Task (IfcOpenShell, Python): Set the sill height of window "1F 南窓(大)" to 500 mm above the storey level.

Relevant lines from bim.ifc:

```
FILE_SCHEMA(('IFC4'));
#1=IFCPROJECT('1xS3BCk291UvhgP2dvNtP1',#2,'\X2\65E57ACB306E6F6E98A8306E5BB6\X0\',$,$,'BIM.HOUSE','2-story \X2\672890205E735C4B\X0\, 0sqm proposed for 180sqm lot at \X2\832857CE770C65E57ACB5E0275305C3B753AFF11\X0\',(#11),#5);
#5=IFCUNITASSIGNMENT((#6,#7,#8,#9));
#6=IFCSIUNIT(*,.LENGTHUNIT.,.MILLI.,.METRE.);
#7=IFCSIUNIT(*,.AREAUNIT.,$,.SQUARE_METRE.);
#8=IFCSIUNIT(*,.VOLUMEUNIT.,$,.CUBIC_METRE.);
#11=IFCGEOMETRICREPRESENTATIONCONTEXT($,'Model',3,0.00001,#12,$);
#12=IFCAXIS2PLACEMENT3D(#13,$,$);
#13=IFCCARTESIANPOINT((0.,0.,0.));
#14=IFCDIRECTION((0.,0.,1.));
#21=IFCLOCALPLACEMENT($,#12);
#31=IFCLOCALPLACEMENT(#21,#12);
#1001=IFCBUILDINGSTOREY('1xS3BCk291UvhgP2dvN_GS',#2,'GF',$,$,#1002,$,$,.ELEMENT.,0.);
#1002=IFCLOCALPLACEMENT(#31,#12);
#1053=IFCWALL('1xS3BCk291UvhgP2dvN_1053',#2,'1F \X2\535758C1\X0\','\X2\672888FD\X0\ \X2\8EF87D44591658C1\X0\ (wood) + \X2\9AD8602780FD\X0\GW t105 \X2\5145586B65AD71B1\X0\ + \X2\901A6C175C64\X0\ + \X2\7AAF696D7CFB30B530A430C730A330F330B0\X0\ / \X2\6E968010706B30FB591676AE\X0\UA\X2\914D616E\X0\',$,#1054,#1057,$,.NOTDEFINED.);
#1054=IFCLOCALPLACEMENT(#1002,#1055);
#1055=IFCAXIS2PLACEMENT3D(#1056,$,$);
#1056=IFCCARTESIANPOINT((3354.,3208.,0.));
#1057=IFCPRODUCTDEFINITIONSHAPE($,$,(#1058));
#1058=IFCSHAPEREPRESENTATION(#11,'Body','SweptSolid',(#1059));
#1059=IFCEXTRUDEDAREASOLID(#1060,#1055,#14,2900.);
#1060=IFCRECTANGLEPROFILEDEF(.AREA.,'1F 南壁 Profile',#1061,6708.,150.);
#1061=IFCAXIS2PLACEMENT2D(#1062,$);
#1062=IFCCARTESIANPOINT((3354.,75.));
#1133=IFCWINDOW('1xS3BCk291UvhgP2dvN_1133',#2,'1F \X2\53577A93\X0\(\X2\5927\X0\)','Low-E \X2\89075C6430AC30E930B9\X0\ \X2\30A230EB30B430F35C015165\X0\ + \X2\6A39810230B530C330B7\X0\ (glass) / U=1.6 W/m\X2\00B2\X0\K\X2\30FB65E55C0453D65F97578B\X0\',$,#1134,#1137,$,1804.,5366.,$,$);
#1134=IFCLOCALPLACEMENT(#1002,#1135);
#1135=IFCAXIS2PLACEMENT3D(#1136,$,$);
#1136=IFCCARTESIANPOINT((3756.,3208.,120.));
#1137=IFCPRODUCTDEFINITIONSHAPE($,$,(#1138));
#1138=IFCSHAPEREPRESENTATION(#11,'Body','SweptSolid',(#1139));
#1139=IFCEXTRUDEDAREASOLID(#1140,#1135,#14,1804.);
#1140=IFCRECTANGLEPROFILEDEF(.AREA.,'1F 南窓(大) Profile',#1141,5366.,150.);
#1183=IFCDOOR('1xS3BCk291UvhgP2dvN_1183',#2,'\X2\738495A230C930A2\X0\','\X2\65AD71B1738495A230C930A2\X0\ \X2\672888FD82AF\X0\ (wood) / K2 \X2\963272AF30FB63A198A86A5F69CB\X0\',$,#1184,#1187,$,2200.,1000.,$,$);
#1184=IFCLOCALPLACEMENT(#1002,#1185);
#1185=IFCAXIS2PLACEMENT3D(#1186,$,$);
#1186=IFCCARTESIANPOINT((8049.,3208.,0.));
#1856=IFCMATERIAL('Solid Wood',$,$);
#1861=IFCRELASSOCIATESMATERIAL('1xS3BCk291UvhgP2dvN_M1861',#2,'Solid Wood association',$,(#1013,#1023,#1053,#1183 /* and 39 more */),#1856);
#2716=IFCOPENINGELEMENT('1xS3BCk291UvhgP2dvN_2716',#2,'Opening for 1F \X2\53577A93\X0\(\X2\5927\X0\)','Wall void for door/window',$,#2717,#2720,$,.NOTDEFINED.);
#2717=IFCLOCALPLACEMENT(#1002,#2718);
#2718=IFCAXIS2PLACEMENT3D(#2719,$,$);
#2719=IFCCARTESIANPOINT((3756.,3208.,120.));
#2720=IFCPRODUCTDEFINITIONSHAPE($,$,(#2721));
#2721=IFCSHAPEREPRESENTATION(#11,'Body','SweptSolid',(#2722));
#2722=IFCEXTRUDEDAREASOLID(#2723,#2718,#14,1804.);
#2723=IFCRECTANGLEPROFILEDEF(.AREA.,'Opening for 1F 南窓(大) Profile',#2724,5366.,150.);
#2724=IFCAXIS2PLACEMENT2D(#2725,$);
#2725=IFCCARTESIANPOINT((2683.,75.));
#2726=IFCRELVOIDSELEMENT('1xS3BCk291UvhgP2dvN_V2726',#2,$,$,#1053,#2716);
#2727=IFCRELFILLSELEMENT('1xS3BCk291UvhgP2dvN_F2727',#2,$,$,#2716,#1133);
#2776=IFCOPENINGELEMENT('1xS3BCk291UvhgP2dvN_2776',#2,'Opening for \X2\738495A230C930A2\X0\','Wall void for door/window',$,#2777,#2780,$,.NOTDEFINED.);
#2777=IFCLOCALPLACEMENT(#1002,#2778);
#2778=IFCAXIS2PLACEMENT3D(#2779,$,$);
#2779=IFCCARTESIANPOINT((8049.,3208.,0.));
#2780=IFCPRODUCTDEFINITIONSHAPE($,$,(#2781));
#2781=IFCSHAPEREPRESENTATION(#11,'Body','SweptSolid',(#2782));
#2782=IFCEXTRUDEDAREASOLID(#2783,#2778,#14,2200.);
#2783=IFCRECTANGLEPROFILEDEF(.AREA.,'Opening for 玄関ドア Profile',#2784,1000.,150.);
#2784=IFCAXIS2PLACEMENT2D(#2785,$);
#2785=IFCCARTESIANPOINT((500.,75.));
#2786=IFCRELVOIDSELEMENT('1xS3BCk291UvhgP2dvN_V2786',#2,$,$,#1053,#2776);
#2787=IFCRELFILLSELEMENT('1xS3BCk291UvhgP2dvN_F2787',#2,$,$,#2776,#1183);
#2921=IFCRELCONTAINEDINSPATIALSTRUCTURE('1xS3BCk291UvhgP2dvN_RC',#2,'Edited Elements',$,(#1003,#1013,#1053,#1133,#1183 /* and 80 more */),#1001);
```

```python
import numpy as np
import ifcopenshell
import ifcopenshell.api.geometry
import ifcopenshell.geom
import ifcopenshell.util.element
import ifcopenshell.util.placement
import ifcopenshell.util.shape
import ifcopenshell.util.unit

model = ifcopenshell.open("bim.ifc")
unit_scale = ifcopenshell.util.unit.calculate_unit_scale(model)

window = model.by_guid("1xS3BCk291UvhgP2dvN_1133")
opening = window.FillsVoids[0].RelatingOpeningElement
storey = ifcopenshell.util.element.get_container(window, ifc_class="IfcBuildingStorey")
level = ifcopenshell.util.placement.get_local_placement(storey.ObjectPlacement)[2, 3]

# The opening's origin need not be at the sill, so measure its lowest point.
shape = ifcopenshell.geom.create_shape(ifcopenshell.geom.settings(), opening)
bottom = ifcopenshell.util.shape.get_shape_bottom_elevation(shape, shape.geometry) / unit_scale
dz = level + 0.5 / unit_scale - bottom

shift = np.array([0.0, 0.0, dz])
# The window is not placed relative to its opening, so move both.
for product in (opening, window):
    matrix = ifcopenshell.util.placement.get_local_placement(product.ObjectPlacement)
    matrix[:3, 3] += shift
    ifcopenshell.api.geometry.edit_object_placement(model, product=product, matrix=matrix, is_si=False)

print(f"moved by {dz * unit_scale:+.3f} m")

model.write("bim_edited.ifc")
```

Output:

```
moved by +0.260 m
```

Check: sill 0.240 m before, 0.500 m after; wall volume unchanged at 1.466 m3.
